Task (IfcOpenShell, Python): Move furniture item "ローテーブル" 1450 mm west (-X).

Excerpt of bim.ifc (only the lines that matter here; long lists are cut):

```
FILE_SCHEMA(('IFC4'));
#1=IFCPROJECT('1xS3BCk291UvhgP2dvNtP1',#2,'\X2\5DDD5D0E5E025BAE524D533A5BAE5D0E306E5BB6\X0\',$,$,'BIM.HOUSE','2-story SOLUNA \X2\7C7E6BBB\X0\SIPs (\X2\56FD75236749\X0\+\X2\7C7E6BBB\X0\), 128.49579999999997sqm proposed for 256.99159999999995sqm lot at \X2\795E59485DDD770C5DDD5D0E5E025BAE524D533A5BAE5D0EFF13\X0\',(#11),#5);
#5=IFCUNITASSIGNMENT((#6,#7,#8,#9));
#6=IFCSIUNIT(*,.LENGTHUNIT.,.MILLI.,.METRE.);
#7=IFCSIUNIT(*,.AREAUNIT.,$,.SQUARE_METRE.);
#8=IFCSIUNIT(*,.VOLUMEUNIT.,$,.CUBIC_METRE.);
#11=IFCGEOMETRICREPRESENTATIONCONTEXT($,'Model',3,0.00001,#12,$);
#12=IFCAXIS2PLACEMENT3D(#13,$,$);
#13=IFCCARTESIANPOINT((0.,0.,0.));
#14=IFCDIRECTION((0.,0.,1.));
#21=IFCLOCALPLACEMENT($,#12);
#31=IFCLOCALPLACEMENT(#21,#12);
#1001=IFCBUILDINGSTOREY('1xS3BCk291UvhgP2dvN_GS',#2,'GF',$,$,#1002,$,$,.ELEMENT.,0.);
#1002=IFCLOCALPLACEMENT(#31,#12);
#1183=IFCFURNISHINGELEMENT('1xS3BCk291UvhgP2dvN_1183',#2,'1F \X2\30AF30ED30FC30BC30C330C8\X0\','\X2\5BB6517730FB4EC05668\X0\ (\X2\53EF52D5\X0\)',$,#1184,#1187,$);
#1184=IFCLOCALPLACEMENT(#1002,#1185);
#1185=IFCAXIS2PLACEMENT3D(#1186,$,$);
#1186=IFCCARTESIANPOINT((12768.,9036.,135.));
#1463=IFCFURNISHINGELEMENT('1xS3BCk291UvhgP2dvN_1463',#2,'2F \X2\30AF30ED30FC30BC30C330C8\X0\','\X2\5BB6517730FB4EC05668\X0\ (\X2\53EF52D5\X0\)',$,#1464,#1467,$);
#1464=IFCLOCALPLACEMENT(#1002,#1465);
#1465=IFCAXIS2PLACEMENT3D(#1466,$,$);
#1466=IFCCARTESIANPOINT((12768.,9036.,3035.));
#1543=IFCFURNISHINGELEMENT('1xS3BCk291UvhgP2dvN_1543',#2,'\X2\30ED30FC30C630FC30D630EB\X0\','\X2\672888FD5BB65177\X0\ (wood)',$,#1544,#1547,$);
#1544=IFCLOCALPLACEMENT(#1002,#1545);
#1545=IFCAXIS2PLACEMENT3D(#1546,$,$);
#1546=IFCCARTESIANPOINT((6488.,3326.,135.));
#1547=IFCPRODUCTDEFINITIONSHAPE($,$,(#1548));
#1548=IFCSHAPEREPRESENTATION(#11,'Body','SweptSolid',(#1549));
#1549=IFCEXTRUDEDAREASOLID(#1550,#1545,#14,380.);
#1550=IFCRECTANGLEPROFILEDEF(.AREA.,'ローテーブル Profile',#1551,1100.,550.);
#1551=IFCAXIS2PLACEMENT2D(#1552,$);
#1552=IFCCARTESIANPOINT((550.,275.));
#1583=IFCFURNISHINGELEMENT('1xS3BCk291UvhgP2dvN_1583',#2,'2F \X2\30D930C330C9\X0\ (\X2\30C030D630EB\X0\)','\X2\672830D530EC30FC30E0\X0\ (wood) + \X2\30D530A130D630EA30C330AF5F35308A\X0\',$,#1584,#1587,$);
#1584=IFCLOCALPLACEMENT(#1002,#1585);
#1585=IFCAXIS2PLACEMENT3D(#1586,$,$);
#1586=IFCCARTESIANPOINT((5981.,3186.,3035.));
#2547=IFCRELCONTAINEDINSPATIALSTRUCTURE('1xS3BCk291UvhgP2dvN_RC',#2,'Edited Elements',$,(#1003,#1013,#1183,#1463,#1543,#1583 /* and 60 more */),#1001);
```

```python
import ifcopenshell
import ifcopenshell.api.geometry
import ifcopenshell.util.placement
import ifcopenshell.util.unit

model = ifcopenshell.open("bim.ifc")
unit_scale = ifcopenshell.util.unit.calculate_unit_scale(model)

item = model.by_guid("1xS3BCk291UvhgP2dvN_1543")
matrix = ifcopenshell.util.placement.get_local_placement(item.ObjectPlacement)
matrix[0, 3] -= 1.45 / unit_scale
ifcopenshell.api.geometry.edit_object_placement(model, product=item, matrix=matrix, is_si=False)

print(ifcopenshell.util.placement.get_local_placement(item.ObjectPlacement).round(3) + 0.0)

model.write("bim_rev.ifc")
```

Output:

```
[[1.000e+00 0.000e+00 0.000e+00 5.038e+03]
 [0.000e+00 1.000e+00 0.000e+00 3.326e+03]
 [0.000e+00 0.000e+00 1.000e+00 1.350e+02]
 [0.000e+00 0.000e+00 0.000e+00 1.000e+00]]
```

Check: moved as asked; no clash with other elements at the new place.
